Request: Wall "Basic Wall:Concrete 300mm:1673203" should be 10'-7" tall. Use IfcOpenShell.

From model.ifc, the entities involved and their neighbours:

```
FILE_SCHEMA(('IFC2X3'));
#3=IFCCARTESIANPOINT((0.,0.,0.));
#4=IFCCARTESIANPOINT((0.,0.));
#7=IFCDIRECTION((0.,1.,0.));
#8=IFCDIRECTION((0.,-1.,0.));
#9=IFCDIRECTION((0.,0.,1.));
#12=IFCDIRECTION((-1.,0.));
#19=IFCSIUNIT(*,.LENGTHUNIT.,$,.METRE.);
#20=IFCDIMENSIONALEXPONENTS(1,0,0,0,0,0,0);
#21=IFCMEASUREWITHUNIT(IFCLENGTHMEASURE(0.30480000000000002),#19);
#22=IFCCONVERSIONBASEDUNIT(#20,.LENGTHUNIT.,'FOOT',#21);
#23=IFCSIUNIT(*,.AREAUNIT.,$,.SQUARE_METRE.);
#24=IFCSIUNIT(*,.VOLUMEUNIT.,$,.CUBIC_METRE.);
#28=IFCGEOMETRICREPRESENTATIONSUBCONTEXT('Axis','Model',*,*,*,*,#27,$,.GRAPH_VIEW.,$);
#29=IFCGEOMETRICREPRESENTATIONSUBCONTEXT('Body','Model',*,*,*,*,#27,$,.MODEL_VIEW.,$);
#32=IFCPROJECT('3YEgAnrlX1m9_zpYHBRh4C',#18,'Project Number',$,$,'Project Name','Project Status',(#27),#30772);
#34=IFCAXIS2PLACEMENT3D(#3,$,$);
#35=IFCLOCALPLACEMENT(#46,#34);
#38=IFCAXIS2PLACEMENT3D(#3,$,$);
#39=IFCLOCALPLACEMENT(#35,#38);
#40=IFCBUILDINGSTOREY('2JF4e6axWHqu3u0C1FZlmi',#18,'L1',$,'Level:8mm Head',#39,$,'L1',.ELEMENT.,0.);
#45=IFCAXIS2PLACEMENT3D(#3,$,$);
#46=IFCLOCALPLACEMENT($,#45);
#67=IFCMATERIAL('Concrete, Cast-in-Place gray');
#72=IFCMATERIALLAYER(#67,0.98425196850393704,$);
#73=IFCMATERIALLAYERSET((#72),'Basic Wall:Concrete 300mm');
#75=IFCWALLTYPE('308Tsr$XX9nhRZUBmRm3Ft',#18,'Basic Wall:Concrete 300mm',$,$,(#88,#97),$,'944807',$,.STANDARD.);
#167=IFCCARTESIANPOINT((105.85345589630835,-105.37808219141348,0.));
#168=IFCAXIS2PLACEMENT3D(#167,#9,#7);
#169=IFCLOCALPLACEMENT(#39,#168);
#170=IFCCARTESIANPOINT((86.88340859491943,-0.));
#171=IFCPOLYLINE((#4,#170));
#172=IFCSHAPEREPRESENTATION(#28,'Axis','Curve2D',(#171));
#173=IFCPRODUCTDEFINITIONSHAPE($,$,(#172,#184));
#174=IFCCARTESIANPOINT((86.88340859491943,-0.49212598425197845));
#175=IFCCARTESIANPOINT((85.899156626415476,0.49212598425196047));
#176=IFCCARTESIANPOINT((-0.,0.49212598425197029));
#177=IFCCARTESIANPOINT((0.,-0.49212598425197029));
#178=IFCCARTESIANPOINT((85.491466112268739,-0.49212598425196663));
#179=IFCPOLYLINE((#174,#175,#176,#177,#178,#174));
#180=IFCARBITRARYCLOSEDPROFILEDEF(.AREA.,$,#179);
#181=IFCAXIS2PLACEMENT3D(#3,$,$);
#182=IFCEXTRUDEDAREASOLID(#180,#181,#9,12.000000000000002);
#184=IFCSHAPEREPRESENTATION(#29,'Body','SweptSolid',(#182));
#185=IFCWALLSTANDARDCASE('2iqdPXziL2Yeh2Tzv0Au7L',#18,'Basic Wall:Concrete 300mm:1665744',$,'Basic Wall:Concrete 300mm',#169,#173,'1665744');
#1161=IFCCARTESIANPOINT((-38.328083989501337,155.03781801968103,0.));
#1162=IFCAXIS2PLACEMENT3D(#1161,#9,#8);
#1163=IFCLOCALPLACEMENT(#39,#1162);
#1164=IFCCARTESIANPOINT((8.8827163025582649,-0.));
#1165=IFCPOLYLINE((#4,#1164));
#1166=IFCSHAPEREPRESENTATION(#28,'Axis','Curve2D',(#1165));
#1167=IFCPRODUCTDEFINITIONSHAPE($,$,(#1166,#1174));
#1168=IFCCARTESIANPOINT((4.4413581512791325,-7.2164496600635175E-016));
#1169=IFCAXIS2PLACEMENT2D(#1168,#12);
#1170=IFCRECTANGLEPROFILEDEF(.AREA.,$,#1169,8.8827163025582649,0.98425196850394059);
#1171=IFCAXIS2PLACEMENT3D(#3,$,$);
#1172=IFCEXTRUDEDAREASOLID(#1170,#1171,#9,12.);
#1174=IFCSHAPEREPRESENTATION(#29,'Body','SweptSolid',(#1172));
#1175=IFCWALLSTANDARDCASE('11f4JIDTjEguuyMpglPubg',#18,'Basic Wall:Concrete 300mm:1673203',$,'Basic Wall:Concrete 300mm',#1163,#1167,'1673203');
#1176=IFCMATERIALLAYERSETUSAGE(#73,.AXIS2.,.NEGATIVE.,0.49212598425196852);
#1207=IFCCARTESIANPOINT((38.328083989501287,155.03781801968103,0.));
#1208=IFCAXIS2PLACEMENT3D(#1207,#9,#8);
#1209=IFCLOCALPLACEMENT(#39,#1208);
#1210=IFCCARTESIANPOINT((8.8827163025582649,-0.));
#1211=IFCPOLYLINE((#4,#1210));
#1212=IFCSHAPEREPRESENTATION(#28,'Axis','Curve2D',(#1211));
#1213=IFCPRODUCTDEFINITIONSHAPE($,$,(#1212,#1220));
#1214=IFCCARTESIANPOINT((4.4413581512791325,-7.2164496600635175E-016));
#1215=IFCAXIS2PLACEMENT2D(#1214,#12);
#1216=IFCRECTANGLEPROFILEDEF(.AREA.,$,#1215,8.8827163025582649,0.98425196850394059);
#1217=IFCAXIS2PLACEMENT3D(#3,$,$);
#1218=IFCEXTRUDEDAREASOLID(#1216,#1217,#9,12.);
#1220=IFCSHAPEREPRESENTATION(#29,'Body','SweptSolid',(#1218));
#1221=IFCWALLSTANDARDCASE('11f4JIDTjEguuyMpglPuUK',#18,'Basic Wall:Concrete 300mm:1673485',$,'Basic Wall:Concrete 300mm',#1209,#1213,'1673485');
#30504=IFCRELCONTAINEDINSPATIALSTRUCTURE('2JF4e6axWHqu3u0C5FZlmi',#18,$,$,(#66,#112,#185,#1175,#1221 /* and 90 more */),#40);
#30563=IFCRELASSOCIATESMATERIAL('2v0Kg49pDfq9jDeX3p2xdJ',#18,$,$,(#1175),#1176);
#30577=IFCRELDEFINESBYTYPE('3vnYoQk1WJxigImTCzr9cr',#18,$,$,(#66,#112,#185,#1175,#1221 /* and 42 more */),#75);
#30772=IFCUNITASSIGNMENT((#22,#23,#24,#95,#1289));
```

```python
import ifcopenshell
import ifcopenshell.geom
import ifcopenshell.util.representation
import ifcopenshell.util.shape
import ifcopenshell.util.unit

model = ifcopenshell.open("model.ifc")
unit_scale = ifcopenshell.util.unit.calculate_unit_scale(model)
settings = ifcopenshell.geom.settings()


def volume(element):
    """Net volume in cubic metres, openings subtracted."""
    shape = ifcopenshell.geom.create_shape(settings, element)
    return ifcopenshell.util.shape.get_volume(shape.geometry)


wall = model.by_guid("11f4JIDTjEguuyMpglPubg")
before = volume(wall)

body = ifcopenshell.util.representation.get_representation(wall, "Model", "Body")
solid = body.Items[0]
old_height = solid.Depth
solid.Depth = 127 * 0.0254 / unit_scale
after = volume(wall)

print(f"height {old_height:g} -> {solid.Depth:g}, volume {before:.3f} -> {after:.3f} m3")

model.write("model_rev.ifc")
```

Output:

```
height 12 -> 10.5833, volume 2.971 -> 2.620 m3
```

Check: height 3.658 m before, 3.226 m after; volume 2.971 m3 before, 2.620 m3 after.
